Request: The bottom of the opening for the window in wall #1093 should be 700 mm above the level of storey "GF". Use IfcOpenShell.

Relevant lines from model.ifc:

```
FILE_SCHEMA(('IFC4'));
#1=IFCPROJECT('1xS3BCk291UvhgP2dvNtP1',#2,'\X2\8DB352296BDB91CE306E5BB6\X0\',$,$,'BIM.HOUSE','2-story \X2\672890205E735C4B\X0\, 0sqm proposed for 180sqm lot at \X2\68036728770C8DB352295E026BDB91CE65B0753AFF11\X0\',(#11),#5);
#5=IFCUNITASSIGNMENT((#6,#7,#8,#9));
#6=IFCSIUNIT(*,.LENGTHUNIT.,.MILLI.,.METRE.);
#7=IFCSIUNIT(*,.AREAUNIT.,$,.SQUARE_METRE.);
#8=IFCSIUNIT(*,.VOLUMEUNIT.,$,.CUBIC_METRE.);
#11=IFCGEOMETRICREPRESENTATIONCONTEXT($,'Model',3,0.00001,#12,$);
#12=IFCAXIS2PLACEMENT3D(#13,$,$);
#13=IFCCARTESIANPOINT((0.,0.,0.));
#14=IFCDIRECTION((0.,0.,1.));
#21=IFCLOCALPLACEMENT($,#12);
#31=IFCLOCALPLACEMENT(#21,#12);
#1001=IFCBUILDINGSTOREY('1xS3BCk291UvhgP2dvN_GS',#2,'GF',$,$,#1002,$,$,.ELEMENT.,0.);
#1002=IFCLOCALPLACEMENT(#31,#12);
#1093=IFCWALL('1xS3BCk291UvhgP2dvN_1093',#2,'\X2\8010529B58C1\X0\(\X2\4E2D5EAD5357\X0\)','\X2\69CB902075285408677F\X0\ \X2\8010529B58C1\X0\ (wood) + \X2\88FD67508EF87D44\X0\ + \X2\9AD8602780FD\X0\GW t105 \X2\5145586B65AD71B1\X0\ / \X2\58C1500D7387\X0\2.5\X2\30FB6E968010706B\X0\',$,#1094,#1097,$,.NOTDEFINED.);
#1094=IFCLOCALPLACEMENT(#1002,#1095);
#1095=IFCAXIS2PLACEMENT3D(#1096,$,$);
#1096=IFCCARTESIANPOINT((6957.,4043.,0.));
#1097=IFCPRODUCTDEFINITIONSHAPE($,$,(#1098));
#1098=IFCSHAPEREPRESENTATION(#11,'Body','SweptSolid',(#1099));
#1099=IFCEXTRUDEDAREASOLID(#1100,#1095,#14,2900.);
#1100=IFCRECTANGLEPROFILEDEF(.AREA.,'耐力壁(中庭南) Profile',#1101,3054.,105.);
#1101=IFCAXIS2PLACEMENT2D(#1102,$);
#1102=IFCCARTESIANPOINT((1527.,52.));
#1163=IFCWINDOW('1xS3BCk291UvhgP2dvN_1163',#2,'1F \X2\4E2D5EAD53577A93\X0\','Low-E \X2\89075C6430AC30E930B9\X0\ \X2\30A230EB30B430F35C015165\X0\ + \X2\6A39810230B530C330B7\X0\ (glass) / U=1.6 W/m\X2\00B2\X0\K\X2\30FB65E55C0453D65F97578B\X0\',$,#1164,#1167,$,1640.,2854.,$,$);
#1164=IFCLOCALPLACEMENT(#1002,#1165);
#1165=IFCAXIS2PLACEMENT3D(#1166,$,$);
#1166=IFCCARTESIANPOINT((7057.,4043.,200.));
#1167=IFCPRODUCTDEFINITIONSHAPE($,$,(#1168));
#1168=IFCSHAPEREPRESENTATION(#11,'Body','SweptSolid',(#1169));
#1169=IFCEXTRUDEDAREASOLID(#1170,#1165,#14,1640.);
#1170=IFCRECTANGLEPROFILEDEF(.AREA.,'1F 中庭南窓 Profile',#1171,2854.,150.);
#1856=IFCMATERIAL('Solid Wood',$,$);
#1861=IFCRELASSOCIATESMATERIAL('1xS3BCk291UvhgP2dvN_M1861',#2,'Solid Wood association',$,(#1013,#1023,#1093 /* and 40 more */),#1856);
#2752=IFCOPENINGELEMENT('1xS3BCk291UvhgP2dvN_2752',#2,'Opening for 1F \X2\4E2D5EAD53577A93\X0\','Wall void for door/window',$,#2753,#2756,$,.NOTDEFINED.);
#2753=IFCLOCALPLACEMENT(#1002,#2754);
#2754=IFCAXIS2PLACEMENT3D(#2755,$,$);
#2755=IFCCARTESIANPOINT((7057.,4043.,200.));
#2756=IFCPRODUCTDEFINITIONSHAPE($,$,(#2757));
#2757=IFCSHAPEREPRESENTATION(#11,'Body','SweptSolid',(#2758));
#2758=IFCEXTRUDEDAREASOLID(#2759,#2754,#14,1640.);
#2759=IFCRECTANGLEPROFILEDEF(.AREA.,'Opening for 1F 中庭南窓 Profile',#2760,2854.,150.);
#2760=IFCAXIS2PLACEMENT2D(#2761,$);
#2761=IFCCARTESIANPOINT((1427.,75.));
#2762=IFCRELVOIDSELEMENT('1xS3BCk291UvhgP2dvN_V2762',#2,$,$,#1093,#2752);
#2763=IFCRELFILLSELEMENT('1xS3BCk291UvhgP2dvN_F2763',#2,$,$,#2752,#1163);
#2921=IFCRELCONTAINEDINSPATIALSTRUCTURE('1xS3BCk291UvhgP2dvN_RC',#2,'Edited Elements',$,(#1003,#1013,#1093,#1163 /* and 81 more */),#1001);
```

```python
import numpy as np
import ifcopenshell
import ifcopenshell.api.geometry
import ifcopenshell.geom
import ifcopenshell.util.element
import ifcopenshell.util.placement
import ifcopenshell.util.shape
import ifcopenshell.util.unit

model = ifcopenshell.open("model.ifc")
unit_scale = ifcopenshell.util.unit.calculate_unit_scale(model)

window = model.by_guid("1xS3BCk291UvhgP2dvN_1163")
opening = window.FillsVoids[0].RelatingOpeningElement
storey = ifcopenshell.util.element.get_container(window, ifc_class="IfcBuildingStorey")
level = ifcopenshell.util.placement.get_local_placement(storey.ObjectPlacement)[2, 3]

# The opening's origin need not be at the sill, so measure its lowest point.
shape = ifcopenshell.geom.create_shape(ifcopenshell.geom.settings(), opening)
bottom = ifcopenshell.util.shape.get_shape_bottom_elevation(shape, shape.geometry) / unit_scale
dz = level + 0.7 / unit_scale - bottom

shift = np.array([0.0, 0.0, dz])
# The window is not placed relative to its opening, so move both.
for product in (opening, window):
    matrix = ifcopenshell.util.placement.get_local_placement(product.ObjectPlacement)
    matrix[:3, 3] += shift
    ifcopenshell.api.geometry.edit_object_placement(model, product=product, matrix=matrix, is_si=False)

print(f"moved by {dz * unit_scale:+.3f} m")

model.write("model-out.ifc")
```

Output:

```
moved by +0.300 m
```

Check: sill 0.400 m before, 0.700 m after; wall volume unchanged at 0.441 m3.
